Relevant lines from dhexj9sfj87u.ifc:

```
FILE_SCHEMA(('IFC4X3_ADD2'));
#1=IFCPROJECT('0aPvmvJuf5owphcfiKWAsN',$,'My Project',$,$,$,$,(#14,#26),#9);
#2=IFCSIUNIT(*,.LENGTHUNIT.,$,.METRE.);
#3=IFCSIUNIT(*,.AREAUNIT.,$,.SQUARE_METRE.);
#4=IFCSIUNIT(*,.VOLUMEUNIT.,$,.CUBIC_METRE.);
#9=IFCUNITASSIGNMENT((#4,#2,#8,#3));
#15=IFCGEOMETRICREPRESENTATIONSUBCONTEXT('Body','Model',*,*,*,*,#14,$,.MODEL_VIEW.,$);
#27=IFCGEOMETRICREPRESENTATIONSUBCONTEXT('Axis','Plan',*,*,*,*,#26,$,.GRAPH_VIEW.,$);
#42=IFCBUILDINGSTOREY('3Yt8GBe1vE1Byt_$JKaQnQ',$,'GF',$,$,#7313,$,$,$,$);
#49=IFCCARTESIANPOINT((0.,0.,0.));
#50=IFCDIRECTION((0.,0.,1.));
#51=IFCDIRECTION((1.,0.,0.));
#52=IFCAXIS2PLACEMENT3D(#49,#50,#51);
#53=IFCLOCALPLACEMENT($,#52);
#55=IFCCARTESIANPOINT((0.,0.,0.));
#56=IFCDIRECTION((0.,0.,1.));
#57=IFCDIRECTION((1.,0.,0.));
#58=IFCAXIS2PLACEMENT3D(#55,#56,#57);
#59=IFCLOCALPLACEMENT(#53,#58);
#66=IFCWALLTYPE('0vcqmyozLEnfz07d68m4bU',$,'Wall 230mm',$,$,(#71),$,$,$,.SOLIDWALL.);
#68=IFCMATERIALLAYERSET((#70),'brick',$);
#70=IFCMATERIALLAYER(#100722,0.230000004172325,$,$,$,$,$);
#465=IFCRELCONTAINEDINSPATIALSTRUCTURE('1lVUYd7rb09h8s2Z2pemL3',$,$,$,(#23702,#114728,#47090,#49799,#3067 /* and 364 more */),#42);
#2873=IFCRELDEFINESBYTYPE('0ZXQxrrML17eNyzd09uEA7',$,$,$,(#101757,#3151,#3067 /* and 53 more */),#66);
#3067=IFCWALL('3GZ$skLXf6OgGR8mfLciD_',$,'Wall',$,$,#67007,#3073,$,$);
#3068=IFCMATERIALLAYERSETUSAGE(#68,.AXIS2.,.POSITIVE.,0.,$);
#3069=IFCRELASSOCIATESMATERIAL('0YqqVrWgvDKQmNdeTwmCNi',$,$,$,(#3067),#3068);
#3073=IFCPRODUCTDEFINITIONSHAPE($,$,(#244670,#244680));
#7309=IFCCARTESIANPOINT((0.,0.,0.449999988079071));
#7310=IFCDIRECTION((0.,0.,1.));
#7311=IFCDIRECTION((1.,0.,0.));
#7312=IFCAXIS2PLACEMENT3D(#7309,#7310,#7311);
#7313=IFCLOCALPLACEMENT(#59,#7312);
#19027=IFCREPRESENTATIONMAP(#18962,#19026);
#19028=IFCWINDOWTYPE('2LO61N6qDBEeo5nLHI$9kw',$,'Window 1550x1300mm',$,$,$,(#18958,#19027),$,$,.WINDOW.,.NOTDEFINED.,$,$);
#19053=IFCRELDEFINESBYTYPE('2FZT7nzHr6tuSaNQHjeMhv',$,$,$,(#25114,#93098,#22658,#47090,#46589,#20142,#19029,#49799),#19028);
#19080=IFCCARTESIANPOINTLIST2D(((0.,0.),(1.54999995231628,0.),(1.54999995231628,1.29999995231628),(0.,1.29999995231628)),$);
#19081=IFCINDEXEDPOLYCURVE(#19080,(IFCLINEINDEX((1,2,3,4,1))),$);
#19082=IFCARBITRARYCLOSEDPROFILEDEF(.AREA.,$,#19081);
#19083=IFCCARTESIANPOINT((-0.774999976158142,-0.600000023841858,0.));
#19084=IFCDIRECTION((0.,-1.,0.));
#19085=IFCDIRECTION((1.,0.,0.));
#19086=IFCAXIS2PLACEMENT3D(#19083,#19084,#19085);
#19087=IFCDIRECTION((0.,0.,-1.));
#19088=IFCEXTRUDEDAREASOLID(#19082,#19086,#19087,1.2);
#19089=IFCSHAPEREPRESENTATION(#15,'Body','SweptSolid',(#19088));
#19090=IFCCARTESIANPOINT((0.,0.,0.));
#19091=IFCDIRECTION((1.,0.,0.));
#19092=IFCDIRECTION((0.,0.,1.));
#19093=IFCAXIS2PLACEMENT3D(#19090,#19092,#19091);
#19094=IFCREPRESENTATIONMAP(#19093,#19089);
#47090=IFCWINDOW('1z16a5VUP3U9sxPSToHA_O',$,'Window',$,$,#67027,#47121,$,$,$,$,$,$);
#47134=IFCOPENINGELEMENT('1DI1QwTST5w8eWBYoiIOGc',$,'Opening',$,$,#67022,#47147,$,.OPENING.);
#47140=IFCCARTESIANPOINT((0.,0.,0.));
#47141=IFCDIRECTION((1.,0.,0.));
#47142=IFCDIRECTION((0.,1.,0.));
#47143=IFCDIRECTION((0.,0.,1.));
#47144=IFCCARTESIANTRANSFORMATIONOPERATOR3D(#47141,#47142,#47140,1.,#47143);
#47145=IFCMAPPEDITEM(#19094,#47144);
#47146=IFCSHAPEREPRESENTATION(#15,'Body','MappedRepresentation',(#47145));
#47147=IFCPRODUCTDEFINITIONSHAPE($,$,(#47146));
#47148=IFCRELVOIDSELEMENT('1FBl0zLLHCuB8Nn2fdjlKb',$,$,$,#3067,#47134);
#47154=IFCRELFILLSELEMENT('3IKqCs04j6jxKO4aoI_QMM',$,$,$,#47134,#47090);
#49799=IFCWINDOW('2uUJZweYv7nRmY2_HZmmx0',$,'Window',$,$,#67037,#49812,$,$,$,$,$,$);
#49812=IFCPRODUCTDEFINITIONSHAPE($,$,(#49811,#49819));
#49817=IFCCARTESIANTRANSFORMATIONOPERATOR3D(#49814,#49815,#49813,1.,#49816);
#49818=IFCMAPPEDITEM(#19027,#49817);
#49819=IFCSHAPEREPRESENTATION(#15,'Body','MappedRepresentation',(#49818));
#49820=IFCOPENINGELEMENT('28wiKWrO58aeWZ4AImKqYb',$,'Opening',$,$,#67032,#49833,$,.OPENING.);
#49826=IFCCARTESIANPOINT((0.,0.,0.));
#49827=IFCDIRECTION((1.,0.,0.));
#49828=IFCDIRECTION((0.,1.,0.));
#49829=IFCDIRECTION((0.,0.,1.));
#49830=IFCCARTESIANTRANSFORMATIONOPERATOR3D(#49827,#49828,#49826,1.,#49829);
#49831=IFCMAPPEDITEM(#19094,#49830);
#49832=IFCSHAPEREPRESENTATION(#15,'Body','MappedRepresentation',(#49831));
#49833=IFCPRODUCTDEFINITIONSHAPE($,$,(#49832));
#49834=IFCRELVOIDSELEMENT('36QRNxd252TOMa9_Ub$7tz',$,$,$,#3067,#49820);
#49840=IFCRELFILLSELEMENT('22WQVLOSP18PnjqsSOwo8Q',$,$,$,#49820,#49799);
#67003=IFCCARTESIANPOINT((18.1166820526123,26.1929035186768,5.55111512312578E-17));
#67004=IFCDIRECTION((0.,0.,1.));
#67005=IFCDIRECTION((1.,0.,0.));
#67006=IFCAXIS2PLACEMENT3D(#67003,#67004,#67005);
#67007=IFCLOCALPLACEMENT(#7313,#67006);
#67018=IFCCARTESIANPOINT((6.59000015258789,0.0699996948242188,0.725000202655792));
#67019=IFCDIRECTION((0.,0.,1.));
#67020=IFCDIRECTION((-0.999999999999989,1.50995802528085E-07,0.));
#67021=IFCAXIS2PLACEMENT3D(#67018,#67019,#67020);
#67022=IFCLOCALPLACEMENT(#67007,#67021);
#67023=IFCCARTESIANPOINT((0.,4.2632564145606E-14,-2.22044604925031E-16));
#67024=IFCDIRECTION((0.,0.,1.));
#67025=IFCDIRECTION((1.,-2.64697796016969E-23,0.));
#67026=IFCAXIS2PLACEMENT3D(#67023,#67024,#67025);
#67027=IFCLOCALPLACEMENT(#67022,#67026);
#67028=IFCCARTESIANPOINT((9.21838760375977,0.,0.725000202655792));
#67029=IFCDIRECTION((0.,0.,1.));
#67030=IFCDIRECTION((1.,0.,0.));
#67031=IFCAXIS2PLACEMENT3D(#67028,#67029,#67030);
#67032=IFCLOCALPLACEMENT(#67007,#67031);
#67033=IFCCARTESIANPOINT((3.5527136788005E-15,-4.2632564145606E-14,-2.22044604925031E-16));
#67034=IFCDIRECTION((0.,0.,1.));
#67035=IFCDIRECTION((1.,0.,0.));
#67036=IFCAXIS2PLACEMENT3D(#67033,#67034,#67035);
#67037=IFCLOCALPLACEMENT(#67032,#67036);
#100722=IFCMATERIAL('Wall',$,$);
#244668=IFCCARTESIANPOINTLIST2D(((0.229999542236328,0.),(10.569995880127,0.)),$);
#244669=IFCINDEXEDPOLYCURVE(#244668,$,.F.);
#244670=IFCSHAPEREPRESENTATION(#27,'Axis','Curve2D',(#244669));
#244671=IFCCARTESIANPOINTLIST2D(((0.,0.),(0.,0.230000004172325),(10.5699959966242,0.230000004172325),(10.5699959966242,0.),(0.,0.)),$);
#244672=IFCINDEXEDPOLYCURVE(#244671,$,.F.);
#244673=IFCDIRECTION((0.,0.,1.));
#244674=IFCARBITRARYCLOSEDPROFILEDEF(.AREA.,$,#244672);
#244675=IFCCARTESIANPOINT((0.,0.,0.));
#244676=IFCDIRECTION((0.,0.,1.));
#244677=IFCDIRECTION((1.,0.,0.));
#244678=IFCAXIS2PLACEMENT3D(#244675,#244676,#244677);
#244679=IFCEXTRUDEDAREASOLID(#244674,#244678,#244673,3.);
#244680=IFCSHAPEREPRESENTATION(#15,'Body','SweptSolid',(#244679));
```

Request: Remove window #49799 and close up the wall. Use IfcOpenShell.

```python
import ifcopenshell
import ifcopenshell.api.feature
import ifcopenshell.api.root
import ifcopenshell.geom
import ifcopenshell.util.shape

model = ifcopenshell.open("dhexj9sfj87u.ifc")
settings = ifcopenshell.geom.settings()


def volume(element):
    """Net volume in cubic metres, openings subtracted."""
    shape = ifcopenshell.geom.create_shape(settings, element)
    return ifcopenshell.util.shape.get_volume(shape.geometry)


window = model.by_guid("2uUJZweYv7nRmY2_HZmmx0")
opening = window.FillsVoids[0].RelatingOpeningElement
wall = opening.VoidsElements[0].RelatingBuildingElement
before = volume(wall)

ifcopenshell.api.root.remove_product(model, product=window)
ifcopenshell.api.feature.remove_feature(model, feature=opening)

after = volume(wall)

print(f"wall volume {before:.3f} -> {after:.3f} m3")

model.write("dhexj9sfj87u_edited.ifc")
```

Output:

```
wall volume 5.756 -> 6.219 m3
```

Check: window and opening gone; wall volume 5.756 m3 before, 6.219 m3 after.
